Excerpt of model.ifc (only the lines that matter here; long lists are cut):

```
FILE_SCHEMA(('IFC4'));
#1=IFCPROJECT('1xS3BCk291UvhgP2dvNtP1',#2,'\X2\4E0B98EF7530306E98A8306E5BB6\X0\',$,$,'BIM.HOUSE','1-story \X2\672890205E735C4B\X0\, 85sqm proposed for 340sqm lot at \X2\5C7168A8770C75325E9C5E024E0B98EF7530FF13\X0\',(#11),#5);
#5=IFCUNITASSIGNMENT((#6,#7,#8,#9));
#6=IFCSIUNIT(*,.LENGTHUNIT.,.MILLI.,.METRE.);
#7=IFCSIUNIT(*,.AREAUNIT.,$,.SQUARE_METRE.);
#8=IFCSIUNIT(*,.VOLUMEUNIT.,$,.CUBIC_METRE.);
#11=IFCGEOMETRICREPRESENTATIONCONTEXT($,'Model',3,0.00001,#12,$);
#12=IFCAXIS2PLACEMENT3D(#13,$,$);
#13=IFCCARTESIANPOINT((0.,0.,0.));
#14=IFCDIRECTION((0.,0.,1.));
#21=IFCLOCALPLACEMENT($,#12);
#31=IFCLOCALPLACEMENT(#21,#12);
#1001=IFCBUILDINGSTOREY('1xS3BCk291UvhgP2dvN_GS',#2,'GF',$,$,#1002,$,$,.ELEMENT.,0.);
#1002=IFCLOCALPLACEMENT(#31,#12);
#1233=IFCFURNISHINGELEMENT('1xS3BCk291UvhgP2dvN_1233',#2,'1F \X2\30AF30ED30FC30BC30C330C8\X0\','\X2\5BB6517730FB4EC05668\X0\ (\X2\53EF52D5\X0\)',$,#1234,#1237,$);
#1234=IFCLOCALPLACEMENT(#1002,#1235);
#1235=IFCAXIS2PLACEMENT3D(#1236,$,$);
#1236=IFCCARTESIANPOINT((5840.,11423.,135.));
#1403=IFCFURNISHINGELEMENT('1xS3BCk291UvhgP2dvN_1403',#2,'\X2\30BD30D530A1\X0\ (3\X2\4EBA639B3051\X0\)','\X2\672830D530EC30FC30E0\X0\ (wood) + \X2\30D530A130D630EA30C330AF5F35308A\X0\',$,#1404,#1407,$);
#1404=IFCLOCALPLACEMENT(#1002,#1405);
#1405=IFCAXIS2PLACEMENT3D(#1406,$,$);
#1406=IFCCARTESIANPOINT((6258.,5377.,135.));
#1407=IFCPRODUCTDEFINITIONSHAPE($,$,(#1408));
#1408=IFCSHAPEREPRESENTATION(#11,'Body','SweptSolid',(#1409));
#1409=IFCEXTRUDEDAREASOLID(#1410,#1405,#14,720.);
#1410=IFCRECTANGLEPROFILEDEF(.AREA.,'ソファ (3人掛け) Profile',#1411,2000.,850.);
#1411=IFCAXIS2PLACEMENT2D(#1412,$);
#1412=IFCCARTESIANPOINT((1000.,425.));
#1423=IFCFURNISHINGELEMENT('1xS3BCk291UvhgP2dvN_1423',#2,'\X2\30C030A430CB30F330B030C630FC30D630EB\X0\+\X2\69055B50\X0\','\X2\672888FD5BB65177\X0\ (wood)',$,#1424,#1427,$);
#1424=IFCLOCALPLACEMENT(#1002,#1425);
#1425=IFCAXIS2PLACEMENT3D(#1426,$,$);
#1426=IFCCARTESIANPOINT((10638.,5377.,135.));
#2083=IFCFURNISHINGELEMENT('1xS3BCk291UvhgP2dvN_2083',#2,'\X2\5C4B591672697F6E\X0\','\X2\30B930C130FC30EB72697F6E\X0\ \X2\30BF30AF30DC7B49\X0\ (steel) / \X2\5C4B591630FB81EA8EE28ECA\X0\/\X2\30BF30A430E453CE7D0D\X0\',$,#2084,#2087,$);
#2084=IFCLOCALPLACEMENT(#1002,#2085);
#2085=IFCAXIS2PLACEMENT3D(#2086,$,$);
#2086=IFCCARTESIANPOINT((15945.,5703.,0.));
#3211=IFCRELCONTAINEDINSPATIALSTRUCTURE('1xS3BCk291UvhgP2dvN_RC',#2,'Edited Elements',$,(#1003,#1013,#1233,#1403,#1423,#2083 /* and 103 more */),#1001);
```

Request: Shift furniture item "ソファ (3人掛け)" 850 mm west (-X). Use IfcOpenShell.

```python
import ifcopenshell
import ifcopenshell.api.geometry
import ifcopenshell.util.placement

model = ifcopenshell.open("model.ifc")

item = model.by_guid("1xS3BCk291UvhgP2dvN_1403")
matrix = ifcopenshell.util.placement.get_local_placement(item.ObjectPlacement)
matrix[0, 3] -= 850.0
ifcopenshell.api.geometry.edit_object_placement(model, product=item, matrix=matrix, is_si=False)

print(ifcopenshell.util.placement.get_local_placement(item.ObjectPlacement).round(3) + 0.0)

model.write("model_edited.ifc")
```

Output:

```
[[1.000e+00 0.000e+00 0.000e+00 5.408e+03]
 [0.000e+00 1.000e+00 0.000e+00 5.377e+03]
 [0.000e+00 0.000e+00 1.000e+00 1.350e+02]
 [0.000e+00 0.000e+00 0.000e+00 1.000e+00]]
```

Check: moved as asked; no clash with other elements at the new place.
